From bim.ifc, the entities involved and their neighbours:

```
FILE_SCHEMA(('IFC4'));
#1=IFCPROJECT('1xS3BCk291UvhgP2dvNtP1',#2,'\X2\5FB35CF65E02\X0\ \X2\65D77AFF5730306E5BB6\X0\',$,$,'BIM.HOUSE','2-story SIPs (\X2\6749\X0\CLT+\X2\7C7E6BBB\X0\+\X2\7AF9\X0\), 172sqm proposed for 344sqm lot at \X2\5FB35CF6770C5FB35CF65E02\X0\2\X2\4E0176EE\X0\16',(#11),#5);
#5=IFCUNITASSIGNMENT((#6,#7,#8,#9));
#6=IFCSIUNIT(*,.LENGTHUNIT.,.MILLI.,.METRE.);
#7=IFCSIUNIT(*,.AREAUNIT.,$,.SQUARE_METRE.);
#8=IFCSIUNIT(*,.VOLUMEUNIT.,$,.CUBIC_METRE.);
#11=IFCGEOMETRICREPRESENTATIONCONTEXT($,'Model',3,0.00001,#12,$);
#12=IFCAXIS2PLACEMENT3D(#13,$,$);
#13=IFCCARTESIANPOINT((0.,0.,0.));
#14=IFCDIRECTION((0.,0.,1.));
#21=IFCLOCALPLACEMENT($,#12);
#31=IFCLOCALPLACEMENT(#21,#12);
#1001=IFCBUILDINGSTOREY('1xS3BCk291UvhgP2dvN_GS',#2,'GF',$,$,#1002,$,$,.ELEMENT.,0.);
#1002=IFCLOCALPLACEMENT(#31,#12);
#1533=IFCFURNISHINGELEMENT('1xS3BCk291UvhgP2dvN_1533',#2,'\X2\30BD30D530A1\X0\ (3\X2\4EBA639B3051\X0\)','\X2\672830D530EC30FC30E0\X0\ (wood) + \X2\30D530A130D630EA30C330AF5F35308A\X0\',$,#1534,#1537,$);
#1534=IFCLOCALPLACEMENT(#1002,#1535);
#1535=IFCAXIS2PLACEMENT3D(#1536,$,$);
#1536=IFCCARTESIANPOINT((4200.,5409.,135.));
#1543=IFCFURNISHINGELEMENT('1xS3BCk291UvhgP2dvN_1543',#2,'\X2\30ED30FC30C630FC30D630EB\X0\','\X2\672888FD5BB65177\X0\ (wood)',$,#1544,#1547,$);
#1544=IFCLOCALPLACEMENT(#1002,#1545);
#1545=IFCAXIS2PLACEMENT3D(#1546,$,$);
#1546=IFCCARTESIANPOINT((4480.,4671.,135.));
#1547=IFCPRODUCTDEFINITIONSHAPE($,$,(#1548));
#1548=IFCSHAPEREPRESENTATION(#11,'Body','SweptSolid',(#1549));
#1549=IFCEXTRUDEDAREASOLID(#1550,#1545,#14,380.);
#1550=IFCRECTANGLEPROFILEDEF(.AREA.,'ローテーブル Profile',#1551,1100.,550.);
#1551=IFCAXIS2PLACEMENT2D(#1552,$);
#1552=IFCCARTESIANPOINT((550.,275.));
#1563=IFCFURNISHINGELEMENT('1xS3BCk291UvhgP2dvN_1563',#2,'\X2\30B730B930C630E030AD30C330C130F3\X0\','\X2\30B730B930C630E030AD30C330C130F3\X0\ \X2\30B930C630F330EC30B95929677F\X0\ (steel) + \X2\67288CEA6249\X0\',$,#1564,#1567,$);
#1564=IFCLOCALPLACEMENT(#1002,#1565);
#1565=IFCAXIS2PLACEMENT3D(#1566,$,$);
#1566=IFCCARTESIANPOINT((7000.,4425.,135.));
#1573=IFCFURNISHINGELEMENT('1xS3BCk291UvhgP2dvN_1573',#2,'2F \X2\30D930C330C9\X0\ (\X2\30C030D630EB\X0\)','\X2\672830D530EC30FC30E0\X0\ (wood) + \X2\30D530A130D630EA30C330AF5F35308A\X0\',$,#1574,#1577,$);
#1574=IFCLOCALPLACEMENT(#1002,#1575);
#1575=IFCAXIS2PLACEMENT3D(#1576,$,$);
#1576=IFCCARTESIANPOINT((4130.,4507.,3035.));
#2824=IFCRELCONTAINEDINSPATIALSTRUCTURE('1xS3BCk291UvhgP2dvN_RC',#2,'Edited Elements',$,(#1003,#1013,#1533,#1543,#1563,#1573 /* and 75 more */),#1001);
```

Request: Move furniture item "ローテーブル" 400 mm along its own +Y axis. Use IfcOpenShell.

```python
import ifcopenshell
import ifcopenshell.api.geometry
import ifcopenshell.util.placement
import ifcopenshell.util.unit

model = ifcopenshell.open("bim.ifc")
unit_scale = ifcopenshell.util.unit.calculate_unit_scale(model)

item = model.by_id(1543)
matrix = ifcopenshell.util.placement.get_local_placement(item.ObjectPlacement)
matrix[:3, 3] += matrix[:3, 1] * 0.4 / unit_scale
ifcopenshell.api.geometry.edit_object_placement(model, product=item, matrix=matrix, is_si=False)

print(ifcopenshell.util.placement.get_local_placement(item.ObjectPlacement).round(3) + 0.0)

model.write("bim_rev.ifc")
```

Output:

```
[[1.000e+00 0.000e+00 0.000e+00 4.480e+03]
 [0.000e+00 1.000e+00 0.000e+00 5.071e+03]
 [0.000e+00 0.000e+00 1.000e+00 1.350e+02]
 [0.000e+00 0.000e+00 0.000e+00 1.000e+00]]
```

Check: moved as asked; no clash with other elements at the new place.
